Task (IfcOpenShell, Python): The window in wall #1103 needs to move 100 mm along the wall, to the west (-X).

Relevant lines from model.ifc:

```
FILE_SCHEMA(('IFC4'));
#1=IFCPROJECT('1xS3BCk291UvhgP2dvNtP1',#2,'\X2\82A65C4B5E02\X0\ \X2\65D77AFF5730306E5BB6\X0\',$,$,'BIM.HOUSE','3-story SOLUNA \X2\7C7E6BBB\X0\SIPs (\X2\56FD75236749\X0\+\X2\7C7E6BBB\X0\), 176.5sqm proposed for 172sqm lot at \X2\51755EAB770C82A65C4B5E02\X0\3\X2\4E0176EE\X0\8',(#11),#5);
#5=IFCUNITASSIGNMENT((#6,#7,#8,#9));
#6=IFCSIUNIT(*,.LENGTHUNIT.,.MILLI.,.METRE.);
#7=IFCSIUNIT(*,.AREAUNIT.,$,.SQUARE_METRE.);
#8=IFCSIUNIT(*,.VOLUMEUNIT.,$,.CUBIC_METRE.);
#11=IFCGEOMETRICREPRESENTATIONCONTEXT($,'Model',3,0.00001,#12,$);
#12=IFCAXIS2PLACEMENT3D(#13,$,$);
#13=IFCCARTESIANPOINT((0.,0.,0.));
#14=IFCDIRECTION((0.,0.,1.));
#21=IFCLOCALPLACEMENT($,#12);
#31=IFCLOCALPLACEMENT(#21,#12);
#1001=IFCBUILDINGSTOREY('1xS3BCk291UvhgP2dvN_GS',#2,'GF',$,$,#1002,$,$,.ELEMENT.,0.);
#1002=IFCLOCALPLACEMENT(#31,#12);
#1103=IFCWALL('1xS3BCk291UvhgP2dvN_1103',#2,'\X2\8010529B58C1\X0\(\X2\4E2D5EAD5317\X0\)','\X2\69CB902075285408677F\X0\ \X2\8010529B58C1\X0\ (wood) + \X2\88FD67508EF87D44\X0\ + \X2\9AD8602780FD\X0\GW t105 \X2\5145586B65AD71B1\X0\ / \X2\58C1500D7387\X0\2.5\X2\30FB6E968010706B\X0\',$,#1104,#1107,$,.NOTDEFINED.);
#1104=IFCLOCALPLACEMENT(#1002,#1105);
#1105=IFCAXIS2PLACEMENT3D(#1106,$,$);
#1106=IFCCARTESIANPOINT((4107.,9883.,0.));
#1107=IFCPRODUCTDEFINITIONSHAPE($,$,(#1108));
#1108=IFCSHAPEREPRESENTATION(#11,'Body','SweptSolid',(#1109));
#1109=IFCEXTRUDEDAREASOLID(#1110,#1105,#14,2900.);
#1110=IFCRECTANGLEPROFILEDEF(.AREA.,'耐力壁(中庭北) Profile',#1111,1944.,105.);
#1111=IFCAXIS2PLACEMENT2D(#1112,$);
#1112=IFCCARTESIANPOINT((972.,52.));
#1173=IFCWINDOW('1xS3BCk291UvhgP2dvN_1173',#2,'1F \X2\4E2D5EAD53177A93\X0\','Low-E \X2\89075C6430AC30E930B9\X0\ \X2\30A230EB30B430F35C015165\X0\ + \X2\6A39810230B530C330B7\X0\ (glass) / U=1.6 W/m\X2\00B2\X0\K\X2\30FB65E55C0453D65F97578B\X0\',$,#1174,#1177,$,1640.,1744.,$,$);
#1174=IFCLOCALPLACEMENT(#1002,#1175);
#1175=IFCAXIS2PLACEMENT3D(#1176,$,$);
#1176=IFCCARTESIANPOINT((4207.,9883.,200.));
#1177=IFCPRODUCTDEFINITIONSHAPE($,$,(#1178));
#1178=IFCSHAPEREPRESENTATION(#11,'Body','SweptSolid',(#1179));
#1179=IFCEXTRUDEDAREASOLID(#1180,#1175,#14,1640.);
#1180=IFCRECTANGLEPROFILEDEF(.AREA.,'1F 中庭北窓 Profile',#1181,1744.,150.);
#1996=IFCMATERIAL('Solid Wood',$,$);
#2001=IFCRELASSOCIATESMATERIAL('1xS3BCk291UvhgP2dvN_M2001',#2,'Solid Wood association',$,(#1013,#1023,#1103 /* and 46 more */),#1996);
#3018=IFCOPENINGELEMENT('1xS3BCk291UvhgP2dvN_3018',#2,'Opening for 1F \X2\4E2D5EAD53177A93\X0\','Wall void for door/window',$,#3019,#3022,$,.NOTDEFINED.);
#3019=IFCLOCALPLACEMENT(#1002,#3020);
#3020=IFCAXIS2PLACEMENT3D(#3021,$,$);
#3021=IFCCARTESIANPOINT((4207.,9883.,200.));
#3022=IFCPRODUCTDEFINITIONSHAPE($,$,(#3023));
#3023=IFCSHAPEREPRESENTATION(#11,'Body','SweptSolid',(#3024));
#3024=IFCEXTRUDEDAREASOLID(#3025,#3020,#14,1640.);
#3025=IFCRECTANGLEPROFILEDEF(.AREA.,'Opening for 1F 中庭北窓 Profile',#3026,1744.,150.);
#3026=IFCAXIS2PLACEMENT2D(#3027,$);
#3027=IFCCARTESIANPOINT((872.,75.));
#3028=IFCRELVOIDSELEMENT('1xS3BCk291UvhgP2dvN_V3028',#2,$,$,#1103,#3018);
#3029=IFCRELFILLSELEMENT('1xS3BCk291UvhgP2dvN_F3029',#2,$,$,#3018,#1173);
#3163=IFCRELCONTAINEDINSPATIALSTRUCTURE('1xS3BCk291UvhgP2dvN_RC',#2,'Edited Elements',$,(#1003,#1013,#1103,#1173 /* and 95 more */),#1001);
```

```python
import ifcopenshell
import ifcopenshell.api.geometry
import ifcopenshell.util.placement
import ifcopenshell.util.unit

model = ifcopenshell.open("model.ifc")
unit_scale = ifcopenshell.util.unit.calculate_unit_scale(model)

window = model.by_guid("1xS3BCk291UvhgP2dvN_1173")
opening = window.FillsVoids[0].RelatingOpeningElement
wall = opening.VoidsElements[0].RelatingBuildingElement

wall_matrix = ifcopenshell.util.placement.get_local_placement(wall.ObjectPlacement)
shift = wall_matrix[:3, 0] * -0.1 / unit_scale
before = ifcopenshell.util.placement.get_local_placement(window.ObjectPlacement)[:3, 3].copy()

# The window is not placed relative to its opening, so move both.
for product in (opening, window):
    matrix = ifcopenshell.util.placement.get_local_placement(product.ObjectPlacement)
    matrix[:3, 3] += shift
    ifcopenshell.api.geometry.edit_object_placement(model, product=product, matrix=matrix, is_si=False)

after = ifcopenshell.util.placement.get_local_placement(window.ObjectPlacement)[:3, 3]
print("window moved by", (after - before).round(3) + 0.0)

model.write("model_v2.ifc")
```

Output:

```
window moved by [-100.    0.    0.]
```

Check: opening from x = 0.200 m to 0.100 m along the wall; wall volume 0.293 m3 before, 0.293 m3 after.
